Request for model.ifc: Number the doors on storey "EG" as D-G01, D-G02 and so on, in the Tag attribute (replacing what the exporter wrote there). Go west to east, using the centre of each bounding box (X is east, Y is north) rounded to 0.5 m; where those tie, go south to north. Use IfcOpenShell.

First a look at what the model holds.

```python
import ifcopenshell
import ifcopenshell.util.element
import ifcopenshell.util.placement

model = ifcopenshell.open("model.ifc")
print(model.schema)
storey = next(s for s in model.by_type("IfcBuildingStorey") if s.Name == "EG")
doors = [e for e in ifcopenshell.util.element.get_decomposition(storey) if e.is_a("IfcDoor")]
for e in sorted(doors, key=lambda e: e.id()):
    origin = ifcopenshell.util.placement.get_local_placement(e.ObjectPlacement)[:3, 3]
    print(e.id(), e.Tag, e.Name, origin.round(2) + 0.0, sep=" | ")
```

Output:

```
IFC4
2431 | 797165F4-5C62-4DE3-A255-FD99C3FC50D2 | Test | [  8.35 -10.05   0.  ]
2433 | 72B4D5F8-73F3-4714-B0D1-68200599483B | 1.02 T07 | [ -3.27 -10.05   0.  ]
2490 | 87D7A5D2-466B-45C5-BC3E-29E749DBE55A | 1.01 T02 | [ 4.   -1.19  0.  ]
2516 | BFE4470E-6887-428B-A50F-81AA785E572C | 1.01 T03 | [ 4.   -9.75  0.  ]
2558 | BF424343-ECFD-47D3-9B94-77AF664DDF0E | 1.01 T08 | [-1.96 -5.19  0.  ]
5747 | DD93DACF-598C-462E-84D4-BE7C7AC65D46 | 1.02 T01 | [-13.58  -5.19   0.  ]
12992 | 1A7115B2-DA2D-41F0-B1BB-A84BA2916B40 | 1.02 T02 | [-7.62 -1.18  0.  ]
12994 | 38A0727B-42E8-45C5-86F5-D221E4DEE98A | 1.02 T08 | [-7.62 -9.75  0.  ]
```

```python
import ifcopenshell
import ifcopenshell.geom
import ifcopenshell.util.element
import ifcopenshell.util.shape

model = ifcopenshell.open("model.ifc")
settings = ifcopenshell.geom.settings()
settings.set("use-world-coords", True)


def centre(element):
    shape = ifcopenshell.geom.create_shape(settings, element)
    return ifcopenshell.util.shape.get_bbox_centroid(shape.geometry)


storey = next(s for s in model.by_type("IfcBuildingStorey") if s.Name == "EG")
doors = [e for e in ifcopenshell.util.element.get_decomposition(storey) if e.is_a("IfcDoor")]

# Insertion points can sit at a corner or the storey origin, so sort by the geometry (in metres).
centres = {e: centre(e) for e in doors}
doors.sort(key=lambda e: (round(centres[e][0] / 0.5), centres[e][1]))

for i, e in enumerate(doors, start=1):
    number = f"D-G{i:02d}"
    e.Tag = number
    print(e.id(), number)

model.write("model-out.ifc")
```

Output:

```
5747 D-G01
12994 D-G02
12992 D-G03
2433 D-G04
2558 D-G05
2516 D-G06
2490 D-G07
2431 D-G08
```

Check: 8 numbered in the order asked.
